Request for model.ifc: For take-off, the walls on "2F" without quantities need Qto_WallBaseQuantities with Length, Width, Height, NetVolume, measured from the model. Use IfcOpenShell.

First a look at what the model holds.

```python
import ifcopenshell
import ifcopenshell.util.element
import ifcopenshell.util.unit

model = ifcopenshell.open("model.ifc")
print(model.schema)
for unit_type in ("LENGTHUNIT", "AREAUNIT", "VOLUMEUNIT"):
    print(unit_type, ifcopenshell.util.unit.calculate_unit_scale(model, unit_type))
storey = next(s for s in model.by_type("IfcBuildingStorey") if s.Name == "2F")
walls = [e for e in ifcopenshell.util.element.get_decomposition(storey) if e.is_a("IfcWall")]
for e in sorted(walls, key=lambda e: e.id()):
    print(e.id(), e.is_a(), e.Name, list(ifcopenshell.util.element.get_psets(e, qtos_only=True)), sep=" | ")
```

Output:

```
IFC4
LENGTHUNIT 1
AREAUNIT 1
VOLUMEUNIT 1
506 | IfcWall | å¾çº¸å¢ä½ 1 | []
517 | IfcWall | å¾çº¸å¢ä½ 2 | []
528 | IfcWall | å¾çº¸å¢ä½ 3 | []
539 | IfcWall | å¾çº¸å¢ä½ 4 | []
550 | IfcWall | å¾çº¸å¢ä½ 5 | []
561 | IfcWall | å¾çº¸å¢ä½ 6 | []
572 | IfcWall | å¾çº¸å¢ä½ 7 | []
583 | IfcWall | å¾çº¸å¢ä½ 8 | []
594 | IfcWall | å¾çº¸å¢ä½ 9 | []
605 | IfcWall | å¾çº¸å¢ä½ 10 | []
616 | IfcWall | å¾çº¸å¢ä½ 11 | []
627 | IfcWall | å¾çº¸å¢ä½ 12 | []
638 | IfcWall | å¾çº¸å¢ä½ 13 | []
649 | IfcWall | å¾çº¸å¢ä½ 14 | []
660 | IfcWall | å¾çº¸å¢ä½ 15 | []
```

```python
import ifcopenshell
import ifcopenshell.api.pset
import ifcopenshell.geom
import ifcopenshell.util.element
import ifcopenshell.util.shape
import ifcopenshell.util.unit

model = ifcopenshell.open("model.ifc")
unit_scale = ifcopenshell.util.unit.calculate_unit_scale(model)
volume_scale = ifcopenshell.util.unit.calculate_unit_scale(model, "VOLUMEUNIT")
settings = ifcopenshell.geom.settings()

storey = next(s for s in model.by_type("IfcBuildingStorey") if s.Name == "2F")
walls = [e for e in ifcopenshell.util.element.get_decomposition(storey) if e.is_a("IfcWall")]

for e in sorted(walls, key=lambda e: e.id()):
    if ifcopenshell.util.element.get_psets(e, qtos_only=True, should_inherit=False):
        continue
    # Geometry comes back in metres, in the element's own axes.
    shape = ifcopenshell.geom.create_shape(settings, e)
    values = {
        "Length": ifcopenshell.util.shape.get_x(shape.geometry) / unit_scale,
        "Width": ifcopenshell.util.shape.get_y(shape.geometry) / unit_scale,
        "Height": ifcopenshell.util.shape.get_z(shape.geometry) / unit_scale,
        "NetVolume": ifcopenshell.util.shape.get_volume(shape.geometry) / volume_scale,
    }
    qto = ifcopenshell.api.pset.add_qto(model, product=e, name="Qto_WallBaseQuantities")
    ifcopenshell.api.pset.edit_qto(model, qto=qto, properties=values)
    print(e.id(), {k: round(v, 3) for k, v in values.items()})

model.write("model_v2.ifc")
```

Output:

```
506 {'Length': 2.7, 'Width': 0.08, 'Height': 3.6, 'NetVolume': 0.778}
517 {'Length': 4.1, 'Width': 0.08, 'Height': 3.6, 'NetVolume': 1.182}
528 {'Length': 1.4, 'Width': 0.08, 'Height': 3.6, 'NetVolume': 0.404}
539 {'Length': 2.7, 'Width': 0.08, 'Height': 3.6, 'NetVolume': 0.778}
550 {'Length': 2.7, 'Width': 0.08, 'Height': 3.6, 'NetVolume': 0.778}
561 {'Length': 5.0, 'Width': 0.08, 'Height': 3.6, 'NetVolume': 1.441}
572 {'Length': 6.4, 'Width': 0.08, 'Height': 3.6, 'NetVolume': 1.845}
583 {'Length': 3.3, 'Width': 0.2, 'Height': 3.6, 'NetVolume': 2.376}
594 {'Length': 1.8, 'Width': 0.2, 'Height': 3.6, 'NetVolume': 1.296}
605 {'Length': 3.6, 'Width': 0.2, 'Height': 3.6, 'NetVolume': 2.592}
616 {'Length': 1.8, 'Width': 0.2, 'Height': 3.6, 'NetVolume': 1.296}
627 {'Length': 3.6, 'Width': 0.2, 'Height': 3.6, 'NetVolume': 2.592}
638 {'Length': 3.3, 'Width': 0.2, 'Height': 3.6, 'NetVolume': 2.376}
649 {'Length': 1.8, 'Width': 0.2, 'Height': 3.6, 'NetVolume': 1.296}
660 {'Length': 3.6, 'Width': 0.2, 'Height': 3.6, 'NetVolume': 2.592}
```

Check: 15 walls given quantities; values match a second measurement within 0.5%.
